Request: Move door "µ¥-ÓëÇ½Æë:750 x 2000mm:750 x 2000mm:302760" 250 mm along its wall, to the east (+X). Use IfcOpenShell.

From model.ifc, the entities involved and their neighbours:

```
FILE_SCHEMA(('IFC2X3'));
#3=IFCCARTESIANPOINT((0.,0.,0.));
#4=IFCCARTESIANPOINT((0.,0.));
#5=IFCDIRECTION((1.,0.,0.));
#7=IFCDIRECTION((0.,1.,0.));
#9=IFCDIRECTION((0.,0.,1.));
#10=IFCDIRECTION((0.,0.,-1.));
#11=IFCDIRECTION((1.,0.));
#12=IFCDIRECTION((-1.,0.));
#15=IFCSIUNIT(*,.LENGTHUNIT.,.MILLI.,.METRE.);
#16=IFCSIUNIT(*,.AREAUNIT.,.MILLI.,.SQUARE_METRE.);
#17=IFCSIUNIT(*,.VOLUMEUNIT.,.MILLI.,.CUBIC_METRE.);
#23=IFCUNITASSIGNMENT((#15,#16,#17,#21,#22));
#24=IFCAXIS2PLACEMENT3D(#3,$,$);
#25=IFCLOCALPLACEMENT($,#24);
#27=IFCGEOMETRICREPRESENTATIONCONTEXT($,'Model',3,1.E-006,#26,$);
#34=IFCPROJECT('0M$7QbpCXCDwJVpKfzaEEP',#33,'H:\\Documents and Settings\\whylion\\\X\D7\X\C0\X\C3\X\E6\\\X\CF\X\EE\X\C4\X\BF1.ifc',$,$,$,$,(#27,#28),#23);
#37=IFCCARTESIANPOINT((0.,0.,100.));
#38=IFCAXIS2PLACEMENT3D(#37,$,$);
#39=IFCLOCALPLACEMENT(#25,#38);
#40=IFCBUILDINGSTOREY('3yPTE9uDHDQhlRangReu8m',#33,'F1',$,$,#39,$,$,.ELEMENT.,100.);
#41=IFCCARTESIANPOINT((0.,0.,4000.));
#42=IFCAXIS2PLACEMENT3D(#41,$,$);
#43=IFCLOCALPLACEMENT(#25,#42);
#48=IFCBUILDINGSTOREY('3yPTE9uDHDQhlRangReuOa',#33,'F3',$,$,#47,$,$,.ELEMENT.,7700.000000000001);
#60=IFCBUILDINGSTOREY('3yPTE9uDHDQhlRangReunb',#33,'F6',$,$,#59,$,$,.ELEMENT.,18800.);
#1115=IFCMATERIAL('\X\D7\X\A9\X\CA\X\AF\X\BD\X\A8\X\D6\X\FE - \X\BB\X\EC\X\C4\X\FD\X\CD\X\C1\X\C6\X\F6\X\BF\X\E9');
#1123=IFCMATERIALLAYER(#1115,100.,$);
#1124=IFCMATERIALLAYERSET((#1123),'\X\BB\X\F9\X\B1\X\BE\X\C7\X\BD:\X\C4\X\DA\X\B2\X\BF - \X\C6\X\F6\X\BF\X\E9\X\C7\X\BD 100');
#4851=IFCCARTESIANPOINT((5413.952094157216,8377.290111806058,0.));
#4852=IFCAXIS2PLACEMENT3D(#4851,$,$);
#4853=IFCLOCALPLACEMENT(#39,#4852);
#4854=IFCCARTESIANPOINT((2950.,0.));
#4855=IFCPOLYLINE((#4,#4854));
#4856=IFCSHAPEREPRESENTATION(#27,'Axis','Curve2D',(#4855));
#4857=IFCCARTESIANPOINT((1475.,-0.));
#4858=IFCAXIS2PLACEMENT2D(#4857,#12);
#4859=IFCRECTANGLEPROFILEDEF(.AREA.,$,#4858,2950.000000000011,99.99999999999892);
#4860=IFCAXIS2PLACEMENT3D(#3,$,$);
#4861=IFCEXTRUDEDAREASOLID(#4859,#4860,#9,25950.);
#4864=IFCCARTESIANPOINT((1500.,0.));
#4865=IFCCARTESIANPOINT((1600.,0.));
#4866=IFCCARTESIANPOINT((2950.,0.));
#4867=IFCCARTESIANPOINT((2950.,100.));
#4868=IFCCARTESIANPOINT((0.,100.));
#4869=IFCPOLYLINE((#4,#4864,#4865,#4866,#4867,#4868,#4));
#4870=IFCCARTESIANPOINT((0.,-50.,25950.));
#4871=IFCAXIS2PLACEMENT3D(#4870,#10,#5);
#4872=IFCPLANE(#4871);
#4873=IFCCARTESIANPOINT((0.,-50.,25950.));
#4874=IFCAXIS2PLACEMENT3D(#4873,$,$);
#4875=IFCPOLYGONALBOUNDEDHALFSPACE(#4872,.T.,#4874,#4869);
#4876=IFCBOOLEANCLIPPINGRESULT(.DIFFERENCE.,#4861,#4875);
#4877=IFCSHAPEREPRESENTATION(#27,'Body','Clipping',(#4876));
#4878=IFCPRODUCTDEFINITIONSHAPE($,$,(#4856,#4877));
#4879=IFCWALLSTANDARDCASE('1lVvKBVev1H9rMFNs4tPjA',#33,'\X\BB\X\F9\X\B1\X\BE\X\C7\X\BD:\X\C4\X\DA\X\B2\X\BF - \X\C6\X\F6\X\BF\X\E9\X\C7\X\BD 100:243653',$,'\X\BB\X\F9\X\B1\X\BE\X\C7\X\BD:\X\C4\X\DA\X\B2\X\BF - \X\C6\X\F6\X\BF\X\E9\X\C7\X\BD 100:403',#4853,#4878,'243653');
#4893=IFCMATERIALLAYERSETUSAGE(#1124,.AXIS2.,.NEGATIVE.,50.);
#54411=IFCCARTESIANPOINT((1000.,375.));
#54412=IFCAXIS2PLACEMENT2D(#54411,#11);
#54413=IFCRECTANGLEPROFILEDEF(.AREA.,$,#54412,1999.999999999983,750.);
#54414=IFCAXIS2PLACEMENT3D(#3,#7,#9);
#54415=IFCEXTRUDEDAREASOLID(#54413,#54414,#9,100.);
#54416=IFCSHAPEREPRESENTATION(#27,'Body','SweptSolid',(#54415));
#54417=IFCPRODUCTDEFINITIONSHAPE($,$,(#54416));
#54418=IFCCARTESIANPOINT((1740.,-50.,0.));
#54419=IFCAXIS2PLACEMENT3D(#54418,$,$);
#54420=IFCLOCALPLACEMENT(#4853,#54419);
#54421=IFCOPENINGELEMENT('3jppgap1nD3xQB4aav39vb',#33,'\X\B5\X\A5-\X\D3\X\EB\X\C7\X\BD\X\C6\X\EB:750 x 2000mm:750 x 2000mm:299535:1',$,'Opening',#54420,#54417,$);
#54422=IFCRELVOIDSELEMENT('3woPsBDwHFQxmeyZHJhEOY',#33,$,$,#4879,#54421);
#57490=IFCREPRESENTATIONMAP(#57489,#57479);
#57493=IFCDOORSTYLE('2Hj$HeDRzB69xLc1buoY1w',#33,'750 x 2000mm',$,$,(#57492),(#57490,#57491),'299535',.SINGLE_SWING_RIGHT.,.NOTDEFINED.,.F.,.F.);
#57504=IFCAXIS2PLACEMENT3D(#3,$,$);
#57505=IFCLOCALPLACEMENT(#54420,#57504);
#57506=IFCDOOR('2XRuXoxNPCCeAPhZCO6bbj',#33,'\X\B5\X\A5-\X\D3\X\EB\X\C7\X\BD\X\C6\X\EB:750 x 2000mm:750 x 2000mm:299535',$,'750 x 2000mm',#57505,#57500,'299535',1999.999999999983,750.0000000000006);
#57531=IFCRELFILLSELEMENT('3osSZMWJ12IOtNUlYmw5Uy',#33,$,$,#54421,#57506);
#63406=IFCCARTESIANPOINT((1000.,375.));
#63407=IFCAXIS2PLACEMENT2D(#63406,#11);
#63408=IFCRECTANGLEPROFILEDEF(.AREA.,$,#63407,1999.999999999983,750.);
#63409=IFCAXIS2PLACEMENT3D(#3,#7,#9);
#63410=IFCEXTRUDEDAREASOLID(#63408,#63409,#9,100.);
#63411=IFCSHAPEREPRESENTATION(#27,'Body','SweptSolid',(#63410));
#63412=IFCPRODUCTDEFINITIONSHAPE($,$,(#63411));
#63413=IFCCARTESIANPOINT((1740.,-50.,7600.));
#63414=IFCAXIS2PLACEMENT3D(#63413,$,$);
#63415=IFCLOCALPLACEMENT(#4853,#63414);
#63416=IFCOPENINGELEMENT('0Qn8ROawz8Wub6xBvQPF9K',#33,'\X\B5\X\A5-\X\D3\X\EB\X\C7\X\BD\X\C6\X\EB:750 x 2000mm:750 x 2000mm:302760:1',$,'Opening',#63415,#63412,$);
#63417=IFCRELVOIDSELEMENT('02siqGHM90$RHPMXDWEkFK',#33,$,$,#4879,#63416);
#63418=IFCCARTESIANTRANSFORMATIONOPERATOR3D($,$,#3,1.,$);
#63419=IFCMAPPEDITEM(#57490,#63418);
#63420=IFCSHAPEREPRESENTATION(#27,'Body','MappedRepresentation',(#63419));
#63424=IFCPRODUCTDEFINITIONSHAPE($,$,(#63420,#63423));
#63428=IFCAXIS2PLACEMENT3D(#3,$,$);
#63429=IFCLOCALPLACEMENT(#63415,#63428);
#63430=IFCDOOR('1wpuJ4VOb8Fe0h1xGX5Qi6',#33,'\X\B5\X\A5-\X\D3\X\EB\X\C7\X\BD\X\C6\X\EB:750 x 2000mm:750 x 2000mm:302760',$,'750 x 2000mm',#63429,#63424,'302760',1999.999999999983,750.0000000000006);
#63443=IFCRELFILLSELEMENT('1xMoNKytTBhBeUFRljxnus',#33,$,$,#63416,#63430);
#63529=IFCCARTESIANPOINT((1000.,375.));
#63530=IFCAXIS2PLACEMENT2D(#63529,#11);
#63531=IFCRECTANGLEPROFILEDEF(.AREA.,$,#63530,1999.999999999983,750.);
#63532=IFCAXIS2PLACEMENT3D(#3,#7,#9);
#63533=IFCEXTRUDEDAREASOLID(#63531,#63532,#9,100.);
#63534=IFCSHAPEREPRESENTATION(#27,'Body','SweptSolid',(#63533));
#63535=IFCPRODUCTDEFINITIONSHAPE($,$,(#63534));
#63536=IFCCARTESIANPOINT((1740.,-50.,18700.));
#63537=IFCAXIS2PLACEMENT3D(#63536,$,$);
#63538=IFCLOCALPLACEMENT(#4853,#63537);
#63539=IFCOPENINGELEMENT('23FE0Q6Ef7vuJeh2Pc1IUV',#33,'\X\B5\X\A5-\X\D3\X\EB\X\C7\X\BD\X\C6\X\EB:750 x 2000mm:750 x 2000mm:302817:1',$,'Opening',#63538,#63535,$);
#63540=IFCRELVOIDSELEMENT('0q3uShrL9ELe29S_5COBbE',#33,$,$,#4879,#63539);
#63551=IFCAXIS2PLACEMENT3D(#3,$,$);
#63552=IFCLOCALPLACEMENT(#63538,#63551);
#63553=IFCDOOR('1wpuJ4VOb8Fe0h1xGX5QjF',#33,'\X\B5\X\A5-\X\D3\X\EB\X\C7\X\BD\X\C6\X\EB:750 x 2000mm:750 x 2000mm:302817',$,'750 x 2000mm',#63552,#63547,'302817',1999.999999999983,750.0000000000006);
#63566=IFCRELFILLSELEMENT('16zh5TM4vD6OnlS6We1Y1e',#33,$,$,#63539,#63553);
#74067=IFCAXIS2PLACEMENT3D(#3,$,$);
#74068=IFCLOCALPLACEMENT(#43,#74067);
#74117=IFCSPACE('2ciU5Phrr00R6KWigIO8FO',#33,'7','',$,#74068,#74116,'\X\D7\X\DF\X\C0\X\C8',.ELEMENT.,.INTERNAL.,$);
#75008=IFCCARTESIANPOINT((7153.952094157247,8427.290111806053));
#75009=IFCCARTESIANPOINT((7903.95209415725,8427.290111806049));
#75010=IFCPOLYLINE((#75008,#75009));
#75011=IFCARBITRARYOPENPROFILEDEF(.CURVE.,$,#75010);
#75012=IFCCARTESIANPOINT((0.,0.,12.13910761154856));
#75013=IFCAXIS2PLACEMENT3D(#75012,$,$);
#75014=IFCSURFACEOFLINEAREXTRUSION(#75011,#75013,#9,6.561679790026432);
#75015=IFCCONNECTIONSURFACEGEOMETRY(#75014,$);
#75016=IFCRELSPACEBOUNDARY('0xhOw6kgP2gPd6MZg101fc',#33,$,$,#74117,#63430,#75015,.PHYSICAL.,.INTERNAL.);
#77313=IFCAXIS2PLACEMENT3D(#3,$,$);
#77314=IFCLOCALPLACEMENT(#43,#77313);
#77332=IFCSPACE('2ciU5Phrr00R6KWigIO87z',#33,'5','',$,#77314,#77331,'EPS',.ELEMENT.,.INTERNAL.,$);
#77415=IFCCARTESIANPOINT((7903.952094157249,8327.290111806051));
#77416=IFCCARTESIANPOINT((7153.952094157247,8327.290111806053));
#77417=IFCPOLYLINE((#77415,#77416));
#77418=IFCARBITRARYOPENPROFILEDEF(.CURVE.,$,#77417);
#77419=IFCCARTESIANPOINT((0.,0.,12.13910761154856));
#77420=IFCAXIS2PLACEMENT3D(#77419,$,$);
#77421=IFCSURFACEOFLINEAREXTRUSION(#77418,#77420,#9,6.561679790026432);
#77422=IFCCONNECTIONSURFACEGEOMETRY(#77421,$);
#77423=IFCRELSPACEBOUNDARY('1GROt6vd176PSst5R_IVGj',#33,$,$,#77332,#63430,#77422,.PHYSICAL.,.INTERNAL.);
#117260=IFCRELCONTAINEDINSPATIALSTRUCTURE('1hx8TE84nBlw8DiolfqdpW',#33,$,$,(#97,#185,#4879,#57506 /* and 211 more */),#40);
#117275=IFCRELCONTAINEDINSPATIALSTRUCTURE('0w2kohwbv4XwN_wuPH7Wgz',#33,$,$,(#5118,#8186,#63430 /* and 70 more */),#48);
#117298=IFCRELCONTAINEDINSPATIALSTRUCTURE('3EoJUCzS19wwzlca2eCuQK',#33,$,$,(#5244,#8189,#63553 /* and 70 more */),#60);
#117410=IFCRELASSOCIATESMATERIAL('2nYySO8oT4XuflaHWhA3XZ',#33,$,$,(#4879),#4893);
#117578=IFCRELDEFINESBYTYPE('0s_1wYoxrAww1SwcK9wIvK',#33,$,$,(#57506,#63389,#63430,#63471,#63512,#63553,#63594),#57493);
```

```python
import numpy as np
import ifcopenshell
import ifcopenshell.api.geometry
import ifcopenshell.util.placement
import ifcopenshell.util.unit

model = ifcopenshell.open("model.ifc")
unit_scale = ifcopenshell.util.unit.calculate_unit_scale(model)

door = model.by_guid("1wpuJ4VOb8Fe0h1xGX5Qi6")
opening = door.FillsVoids[0].RelatingOpeningElement
wall = opening.VoidsElements[0].RelatingBuildingElement

wall_matrix = ifcopenshell.util.placement.get_local_placement(wall.ObjectPlacement)
shift = wall_matrix[:3, 0] * 0.25 / unit_scale
before = ifcopenshell.util.placement.get_local_placement(door.ObjectPlacement)[:3, 3].copy()

# The door is placed relative to its opening, so it follows when the opening moves.
matrix = ifcopenshell.util.placement.get_local_placement(opening.ObjectPlacement)
matrix[:3, 3] += shift
ifcopenshell.api.geometry.edit_object_placement(
    model, product=opening, matrix=matrix, is_si=False, should_transform_children=True
)

# Space boundary surfaces are stored in each space's coordinates; move them too.
for rel in door.ProvidesBoundaries:
    if not rel.ConnectionGeometry:
        continue
    surface = rel.ConnectionGeometry.SurfaceOnRelatingElement
    space_matrix = ifcopenshell.util.placement.get_local_placement(rel.RelatingSpace.ObjectPlacement)
    point = np.array(surface.Position.Location.Coordinates) + space_matrix[:3, :3].T @ shift
    surface.Position = model.createIfcAxis2Placement3D(
        model.createIfcCartesianPoint(point.tolist()), surface.Position.Axis, surface.Position.RefDirection
    )

after = ifcopenshell.util.placement.get_local_placement(door.ObjectPlacement)[:3, 3]
print("door moved by", (after - before).round(3) + 0.0)

model.write("model_updated.ifc")
```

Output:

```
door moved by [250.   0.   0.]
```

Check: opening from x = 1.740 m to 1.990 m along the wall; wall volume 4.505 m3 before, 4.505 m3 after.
